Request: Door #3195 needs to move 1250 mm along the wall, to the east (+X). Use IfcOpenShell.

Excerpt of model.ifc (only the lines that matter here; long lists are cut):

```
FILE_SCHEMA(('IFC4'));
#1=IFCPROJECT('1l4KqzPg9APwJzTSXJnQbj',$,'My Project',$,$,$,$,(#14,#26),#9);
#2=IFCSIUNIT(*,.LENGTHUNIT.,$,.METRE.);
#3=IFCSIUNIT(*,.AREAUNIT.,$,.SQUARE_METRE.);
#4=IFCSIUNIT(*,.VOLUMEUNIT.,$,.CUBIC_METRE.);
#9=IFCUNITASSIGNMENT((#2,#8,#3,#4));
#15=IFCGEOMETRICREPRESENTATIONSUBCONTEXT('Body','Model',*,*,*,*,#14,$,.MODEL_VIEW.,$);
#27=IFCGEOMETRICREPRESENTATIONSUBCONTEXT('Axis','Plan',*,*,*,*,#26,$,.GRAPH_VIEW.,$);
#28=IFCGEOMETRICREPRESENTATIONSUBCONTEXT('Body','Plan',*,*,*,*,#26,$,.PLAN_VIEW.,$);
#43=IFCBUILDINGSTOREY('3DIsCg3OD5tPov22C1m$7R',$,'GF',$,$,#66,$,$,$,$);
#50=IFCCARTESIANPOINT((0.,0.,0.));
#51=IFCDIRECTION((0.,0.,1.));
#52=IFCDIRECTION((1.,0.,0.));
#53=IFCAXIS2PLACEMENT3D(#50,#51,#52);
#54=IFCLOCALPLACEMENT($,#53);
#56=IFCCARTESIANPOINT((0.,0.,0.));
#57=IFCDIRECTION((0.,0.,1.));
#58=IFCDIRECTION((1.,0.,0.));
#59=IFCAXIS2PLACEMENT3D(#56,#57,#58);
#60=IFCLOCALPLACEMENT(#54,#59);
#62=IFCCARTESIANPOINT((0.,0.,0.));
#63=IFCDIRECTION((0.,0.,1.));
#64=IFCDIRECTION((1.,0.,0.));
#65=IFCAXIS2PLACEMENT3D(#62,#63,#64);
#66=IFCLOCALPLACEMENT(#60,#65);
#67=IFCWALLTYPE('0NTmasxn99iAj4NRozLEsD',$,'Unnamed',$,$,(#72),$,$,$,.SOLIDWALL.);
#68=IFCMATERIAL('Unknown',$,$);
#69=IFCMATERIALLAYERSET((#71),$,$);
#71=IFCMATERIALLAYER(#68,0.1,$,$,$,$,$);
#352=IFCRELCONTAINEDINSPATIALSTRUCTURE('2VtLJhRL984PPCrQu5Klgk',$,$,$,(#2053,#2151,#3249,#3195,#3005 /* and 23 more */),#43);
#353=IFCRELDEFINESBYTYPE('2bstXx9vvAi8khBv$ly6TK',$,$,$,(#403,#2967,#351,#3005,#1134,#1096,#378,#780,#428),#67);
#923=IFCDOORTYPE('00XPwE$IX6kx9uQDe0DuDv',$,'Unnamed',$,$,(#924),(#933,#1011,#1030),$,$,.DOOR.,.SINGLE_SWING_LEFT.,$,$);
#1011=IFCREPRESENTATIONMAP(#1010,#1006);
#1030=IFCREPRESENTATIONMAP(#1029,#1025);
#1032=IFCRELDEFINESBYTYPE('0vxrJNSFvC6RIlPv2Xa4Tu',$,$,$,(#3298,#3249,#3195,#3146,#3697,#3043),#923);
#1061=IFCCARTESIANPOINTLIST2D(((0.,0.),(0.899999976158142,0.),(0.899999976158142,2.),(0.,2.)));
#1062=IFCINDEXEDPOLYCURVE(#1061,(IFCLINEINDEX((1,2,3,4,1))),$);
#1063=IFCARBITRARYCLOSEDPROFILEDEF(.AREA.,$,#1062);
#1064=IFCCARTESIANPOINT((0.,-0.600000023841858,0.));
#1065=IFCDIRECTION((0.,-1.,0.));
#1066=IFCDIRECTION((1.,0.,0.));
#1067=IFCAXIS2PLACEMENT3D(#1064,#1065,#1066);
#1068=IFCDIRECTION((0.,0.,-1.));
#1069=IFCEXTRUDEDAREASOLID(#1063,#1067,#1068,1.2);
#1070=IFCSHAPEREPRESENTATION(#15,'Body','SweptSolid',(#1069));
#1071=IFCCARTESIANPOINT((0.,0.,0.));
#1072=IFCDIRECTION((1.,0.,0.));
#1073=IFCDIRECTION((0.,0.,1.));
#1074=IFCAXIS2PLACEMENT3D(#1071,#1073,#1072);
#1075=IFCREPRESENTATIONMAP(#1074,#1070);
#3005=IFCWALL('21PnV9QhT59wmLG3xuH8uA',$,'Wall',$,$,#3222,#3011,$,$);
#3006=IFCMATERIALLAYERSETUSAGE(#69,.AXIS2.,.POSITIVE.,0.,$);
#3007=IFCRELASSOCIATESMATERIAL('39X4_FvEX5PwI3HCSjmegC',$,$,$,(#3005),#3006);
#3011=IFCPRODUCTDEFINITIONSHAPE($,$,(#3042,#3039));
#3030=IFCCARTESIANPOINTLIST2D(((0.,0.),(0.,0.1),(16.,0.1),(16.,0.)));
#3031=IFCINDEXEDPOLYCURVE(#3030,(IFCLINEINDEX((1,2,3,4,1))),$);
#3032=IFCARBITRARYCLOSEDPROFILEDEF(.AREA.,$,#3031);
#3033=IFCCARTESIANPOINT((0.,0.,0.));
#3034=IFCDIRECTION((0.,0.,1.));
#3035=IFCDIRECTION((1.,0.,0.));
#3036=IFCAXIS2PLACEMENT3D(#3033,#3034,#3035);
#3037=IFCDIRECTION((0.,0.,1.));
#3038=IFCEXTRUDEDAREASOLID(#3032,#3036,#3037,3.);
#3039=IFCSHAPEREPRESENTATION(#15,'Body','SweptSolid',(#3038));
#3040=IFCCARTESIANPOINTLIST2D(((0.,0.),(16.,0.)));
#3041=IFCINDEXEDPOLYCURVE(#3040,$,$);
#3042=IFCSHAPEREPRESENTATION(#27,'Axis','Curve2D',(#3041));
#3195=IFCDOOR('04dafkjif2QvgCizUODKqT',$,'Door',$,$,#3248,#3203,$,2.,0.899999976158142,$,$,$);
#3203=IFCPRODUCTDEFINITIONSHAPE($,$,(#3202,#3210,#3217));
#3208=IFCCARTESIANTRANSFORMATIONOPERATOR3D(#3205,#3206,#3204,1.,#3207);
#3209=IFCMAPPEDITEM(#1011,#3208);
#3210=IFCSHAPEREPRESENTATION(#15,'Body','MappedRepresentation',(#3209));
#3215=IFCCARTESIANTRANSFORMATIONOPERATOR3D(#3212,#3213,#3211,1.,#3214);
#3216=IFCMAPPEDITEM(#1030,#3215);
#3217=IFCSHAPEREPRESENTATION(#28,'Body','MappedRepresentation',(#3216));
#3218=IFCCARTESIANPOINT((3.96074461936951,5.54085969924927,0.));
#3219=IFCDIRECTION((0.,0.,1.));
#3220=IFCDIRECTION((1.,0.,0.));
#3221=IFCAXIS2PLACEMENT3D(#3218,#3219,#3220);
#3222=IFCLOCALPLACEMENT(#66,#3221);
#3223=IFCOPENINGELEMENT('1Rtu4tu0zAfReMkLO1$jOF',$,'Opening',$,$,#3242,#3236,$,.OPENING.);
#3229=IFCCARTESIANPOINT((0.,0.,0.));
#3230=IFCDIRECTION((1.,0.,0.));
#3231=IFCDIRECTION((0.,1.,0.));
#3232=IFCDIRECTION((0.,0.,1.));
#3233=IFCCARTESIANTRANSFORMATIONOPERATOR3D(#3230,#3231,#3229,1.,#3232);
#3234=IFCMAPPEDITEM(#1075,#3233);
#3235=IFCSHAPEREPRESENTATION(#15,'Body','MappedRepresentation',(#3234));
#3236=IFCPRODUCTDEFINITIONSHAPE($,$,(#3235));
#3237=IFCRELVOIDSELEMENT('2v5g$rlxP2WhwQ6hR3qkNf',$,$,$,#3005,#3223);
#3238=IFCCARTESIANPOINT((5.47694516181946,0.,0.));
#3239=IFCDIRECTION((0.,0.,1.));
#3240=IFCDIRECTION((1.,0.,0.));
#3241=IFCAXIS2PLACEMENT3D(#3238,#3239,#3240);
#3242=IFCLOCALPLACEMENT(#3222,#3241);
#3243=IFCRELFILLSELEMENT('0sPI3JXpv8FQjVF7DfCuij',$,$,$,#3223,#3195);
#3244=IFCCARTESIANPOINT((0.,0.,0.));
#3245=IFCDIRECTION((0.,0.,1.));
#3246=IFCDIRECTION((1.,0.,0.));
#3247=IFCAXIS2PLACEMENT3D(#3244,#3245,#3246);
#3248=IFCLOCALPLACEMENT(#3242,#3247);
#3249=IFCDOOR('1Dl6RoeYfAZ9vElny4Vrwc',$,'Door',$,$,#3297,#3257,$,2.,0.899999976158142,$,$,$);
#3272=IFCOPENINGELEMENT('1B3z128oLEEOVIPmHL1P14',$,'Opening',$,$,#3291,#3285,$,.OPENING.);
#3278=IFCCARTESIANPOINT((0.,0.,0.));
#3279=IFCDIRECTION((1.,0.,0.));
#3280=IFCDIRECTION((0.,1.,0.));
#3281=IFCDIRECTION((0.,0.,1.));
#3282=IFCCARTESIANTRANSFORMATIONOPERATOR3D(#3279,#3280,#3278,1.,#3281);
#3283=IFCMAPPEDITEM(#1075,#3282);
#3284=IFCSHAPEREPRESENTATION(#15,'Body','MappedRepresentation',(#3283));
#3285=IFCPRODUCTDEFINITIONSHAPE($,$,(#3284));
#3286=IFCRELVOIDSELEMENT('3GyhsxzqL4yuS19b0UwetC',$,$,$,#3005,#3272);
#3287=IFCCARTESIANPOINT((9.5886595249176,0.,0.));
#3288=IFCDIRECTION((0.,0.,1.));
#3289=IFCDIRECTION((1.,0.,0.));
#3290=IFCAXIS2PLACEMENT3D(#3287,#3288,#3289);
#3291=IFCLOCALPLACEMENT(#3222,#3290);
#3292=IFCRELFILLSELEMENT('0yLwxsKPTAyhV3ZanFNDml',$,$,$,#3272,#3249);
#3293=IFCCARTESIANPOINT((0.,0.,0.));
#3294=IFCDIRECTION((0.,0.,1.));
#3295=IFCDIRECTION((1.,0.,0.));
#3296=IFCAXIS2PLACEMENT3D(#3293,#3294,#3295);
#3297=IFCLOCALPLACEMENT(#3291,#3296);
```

```python
import ifcopenshell
import ifcopenshell.api.geometry
import ifcopenshell.util.placement

model = ifcopenshell.open("model.ifc")

door = model.by_guid("04dafkjif2QvgCizUODKqT")
opening = door.FillsVoids[0].RelatingOpeningElement
wall = opening.VoidsElements[0].RelatingBuildingElement

wall_matrix = ifcopenshell.util.placement.get_local_placement(wall.ObjectPlacement)
shift = wall_matrix[:3, 0] * 1.25
before = ifcopenshell.util.placement.get_local_placement(door.ObjectPlacement)[:3, 3].copy()

# The door is placed relative to its opening, so it follows when the opening moves.
matrix = ifcopenshell.util.placement.get_local_placement(opening.ObjectPlacement)
matrix[:3, 3] += shift
ifcopenshell.api.geometry.edit_object_placement(
    model, product=opening, matrix=matrix, is_si=False, should_transform_children=True
)

after = ifcopenshell.util.placement.get_local_placement(door.ObjectPlacement)[:3, 3]
print("door moved by", (after - before).round(3) + 0.0)

model.write("model_updated.ifc")
```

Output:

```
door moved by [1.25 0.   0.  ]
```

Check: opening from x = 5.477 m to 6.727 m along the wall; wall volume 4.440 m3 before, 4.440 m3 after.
